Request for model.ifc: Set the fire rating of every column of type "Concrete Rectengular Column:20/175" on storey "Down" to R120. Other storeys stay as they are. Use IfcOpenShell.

First a look at what the model holds.

```python
import ifcopenshell
import ifcopenshell.util.element

model = ifcopenshell.open("model.ifc")
print(model.schema)
storey = next(s for s in model.by_type("IfcBuildingStorey") if s.Name == "Down")
columns = [e for e in ifcopenshell.util.element.get_decomposition(storey) if e.is_a("IfcColumn")]
seen = {}
for e in columns:
    element_type = ifcopenshell.util.element.get_type(e)
    key = (element_type.Name if element_type != e and element_type else None, ifcopenshell.util.element.get_pset(e, "Pset_ColumnCommon", "FireRating"))
    seen[key] = seen.get(key, 0) + 1
for (name, value), count in sorted(seen.items(), key=str):
    print(count, "x", name, "|", value)
```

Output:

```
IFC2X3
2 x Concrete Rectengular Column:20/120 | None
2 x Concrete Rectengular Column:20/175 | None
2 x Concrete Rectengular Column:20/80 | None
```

```python
import ifcopenshell
import ifcopenshell.api.pset
import ifcopenshell.util.element

model = ifcopenshell.open("model.ifc")

storey = next(s for s in model.by_type("IfcBuildingStorey") if s.Name == "Down")
columns = [e for e in ifcopenshell.util.element.get_decomposition(storey) if e.is_a("IfcColumn")]

count = 0
for e in columns:
    element_type = ifcopenshell.util.element.get_type(e)
    if element_type in (None, e) or element_type.Name != "Concrete Rectengular Column:20/175":
        continue
    # add_pset returns the element's existing set when there is one.
    pset = ifcopenshell.api.pset.add_pset(model, product=e, name="Pset_ColumnCommon")
    ifcopenshell.api.pset.edit_pset(model, pset=pset, properties={"FireRating": "R120"})
    count += 1

print(count, "columns updated")

model.write("model_rev.ifc")
```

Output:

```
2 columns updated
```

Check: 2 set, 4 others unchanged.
